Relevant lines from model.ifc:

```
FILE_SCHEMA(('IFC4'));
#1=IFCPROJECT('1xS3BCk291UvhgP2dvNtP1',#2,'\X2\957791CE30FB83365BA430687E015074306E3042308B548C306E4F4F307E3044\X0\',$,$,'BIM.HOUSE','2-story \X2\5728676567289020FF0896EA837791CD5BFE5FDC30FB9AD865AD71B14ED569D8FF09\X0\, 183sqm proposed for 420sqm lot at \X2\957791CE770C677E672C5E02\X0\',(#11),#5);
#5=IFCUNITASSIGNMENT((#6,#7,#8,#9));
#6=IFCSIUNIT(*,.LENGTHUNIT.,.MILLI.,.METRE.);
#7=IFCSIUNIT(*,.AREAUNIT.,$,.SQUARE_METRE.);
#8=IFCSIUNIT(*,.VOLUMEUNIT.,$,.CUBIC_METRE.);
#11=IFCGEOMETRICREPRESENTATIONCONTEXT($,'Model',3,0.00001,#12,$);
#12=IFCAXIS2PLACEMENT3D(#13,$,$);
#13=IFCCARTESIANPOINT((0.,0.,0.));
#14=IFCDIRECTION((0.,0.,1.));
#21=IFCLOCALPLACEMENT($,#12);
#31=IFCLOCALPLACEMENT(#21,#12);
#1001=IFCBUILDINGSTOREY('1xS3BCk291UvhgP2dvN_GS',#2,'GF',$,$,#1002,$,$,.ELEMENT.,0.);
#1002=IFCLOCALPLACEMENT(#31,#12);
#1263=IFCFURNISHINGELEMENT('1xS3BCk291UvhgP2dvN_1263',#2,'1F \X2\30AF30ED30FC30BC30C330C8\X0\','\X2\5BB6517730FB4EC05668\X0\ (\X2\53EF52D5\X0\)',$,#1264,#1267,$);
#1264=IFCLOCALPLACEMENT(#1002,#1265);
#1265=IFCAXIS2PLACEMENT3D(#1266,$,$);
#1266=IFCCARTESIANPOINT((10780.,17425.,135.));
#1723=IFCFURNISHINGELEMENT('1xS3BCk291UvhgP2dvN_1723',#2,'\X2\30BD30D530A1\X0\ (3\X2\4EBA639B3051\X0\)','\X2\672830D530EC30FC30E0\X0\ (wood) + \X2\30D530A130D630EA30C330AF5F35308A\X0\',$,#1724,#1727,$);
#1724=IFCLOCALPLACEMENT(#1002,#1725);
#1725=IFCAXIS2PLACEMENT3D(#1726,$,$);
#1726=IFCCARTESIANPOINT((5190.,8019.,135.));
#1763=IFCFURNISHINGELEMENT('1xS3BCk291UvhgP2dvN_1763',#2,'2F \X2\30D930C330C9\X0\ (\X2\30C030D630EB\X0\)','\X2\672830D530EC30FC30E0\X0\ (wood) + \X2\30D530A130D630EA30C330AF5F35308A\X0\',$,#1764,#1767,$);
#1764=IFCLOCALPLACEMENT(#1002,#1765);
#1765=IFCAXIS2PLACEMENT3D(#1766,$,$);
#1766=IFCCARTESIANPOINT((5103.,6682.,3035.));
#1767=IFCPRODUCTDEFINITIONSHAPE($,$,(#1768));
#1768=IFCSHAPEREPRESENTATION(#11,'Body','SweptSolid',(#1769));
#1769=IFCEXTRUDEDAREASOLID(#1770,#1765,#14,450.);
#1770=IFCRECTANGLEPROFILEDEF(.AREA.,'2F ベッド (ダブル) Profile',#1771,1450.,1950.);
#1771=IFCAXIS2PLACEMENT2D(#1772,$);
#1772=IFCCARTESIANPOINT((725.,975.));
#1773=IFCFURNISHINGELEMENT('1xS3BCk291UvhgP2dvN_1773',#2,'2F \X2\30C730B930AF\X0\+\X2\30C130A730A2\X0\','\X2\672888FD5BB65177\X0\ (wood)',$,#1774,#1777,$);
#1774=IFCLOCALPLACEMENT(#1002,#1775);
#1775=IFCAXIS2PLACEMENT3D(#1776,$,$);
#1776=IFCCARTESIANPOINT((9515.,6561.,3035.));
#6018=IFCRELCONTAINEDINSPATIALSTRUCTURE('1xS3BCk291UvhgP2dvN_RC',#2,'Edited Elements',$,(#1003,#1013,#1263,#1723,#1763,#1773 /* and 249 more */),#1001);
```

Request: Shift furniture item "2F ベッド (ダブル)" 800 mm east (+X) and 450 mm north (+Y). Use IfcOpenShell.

```python
import ifcopenshell
import ifcopenshell.api.geometry
import ifcopenshell.util.placement

model = ifcopenshell.open("model.ifc")

item = model.by_guid("1xS3BCk291UvhgP2dvN_1763")
matrix = ifcopenshell.util.placement.get_local_placement(item.ObjectPlacement)
matrix[0, 3] += 800.0
matrix[1, 3] += 450.0
ifcopenshell.api.geometry.edit_object_placement(model, product=item, matrix=matrix, is_si=False)

print(ifcopenshell.util.placement.get_local_placement(item.ObjectPlacement).round(3) + 0.0)

model.write("model_rev.ifc")
```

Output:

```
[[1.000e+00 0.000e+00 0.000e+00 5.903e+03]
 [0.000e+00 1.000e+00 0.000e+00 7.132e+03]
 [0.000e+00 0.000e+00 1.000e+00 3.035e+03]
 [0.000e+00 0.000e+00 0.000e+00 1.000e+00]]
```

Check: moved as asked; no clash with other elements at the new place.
